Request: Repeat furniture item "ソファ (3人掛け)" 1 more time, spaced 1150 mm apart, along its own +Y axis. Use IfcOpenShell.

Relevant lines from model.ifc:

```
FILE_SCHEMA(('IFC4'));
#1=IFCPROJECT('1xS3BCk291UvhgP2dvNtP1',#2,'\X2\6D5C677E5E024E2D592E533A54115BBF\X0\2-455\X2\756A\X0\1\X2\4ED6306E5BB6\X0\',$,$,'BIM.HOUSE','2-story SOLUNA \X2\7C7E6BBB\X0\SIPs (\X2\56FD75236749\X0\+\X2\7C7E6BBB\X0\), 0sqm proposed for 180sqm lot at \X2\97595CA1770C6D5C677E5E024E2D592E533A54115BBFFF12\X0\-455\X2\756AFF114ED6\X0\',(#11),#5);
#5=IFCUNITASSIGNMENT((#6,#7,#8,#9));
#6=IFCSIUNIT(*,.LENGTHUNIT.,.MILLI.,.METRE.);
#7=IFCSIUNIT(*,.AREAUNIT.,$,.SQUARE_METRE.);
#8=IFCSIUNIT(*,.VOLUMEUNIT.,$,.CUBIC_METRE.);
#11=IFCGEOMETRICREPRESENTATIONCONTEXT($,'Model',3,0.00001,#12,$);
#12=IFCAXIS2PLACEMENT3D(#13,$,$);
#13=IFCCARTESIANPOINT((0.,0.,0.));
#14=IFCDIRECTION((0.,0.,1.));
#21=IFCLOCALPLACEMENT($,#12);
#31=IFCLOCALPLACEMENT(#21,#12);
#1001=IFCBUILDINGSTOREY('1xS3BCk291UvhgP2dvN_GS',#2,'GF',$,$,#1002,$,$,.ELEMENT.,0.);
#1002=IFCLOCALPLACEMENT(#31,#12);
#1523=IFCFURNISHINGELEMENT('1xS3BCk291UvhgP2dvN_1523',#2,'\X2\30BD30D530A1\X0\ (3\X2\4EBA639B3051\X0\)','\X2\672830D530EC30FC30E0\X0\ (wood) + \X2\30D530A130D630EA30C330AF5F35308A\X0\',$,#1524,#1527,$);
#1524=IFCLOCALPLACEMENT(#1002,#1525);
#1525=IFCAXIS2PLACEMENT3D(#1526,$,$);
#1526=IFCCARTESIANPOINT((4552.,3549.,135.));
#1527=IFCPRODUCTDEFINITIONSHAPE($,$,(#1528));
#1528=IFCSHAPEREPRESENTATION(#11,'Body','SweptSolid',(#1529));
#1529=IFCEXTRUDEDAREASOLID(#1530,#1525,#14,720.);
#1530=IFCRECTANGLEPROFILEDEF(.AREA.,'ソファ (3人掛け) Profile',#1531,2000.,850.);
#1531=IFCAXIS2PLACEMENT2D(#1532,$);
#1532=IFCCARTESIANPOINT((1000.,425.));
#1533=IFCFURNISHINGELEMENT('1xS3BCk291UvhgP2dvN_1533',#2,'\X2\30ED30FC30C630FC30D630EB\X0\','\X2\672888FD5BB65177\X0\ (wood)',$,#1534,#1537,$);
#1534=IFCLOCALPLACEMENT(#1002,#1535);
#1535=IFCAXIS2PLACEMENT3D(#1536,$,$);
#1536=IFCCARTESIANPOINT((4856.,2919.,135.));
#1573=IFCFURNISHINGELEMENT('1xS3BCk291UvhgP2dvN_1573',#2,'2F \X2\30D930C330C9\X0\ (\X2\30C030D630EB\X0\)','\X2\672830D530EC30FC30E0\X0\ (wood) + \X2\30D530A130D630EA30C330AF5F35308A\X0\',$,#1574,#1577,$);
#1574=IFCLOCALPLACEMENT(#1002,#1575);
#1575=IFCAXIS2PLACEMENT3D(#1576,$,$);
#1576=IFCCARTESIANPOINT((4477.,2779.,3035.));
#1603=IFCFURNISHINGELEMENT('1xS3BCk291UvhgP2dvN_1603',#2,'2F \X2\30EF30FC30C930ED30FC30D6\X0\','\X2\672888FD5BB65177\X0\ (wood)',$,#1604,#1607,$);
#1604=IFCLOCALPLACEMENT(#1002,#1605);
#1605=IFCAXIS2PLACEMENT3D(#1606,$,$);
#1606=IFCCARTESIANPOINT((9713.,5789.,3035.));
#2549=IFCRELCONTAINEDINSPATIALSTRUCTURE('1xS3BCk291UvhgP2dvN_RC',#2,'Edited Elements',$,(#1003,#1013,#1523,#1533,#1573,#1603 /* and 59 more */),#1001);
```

```python
import ifcopenshell
import ifcopenshell.api.geometry
import ifcopenshell.api.root
import ifcopenshell.util.element
import ifcopenshell.util.placement

model = ifcopenshell.open("model.ifc")


def reuse_history(source, copy):
    """copy_class also copies each property set's owner history, people and application; keep the originals."""
    for rel in copy.IsDefinedBy:
        if rel.is_a("IfcRelDefinesByProperties") and (history := rel.RelatingPropertyDefinition.OwnerHistory):
            rel.RelatingPropertyDefinition.OwnerHistory = source.OwnerHistory
            ifcopenshell.util.element.remove_deep2(model, history)


source = model.by_guid("1xS3BCk291UvhgP2dvN_1523")
base = ifcopenshell.util.placement.get_local_placement(source.ObjectPlacement)
step = base[:3, 1] * 1150.0

for i in range(1, 2):
    copy = ifcopenshell.api.root.copy_class(model, product=source)
    copy.Representation = ifcopenshell.util.element.copy_deep(
        model, source.Representation, exclude=["IfcGeometricRepresentationContext", "IfcRepresentationMap"]
    )
    reuse_history(source, copy)
    matrix = base.copy()
    matrix[:3, 3] += i * step
    print("added at", matrix[:3, 3].round(3) + 0.0)
    ifcopenshell.api.geometry.edit_object_placement(model, product=copy, matrix=matrix, is_si=False)

model.write("model_edited.ifc")
```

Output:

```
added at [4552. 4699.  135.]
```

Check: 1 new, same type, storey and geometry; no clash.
